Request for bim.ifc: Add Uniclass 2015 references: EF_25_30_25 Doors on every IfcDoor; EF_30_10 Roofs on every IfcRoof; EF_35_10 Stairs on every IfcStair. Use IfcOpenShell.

First a look at what the model holds.

```python
import ifcopenshell

model = ifcopenshell.open("bim.ifc")
print(model.schema)
print("classifications:", [c.Name for c in model.by_type("IfcClassification")])
for ifc_class in ("IfcDoor", "IfcRoof", "IfcStair", "IfcWall", "IfcWindow"):
    print(ifc_class, len(model.by_type(ifc_class)))
```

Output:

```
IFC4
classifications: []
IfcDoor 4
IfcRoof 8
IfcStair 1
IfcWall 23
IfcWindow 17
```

```python
import ifcopenshell
import ifcopenshell.api.classification

model = ifcopenshell.open("bim.ifc")

system = ifcopenshell.api.classification.add_classification(model, classification="Uniclass 2015")

codes = {
    "IfcDoor": ("EF_25_30_25", "Doors"),
    "IfcRoof": ("EF_30_10", "Roofs"),
    "IfcStair": ("EF_35_10", "Stairs"),
}
for ifc_class, (code, name) in codes.items():
    products = model.by_type(ifc_class)
    ifcopenshell.api.classification.add_reference(
        model, products=products, classification=system, identification=code, name=name
    )
    print(code, len(products))

model.write("bim_edited.ifc")
```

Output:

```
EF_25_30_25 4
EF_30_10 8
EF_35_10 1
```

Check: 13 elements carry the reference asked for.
